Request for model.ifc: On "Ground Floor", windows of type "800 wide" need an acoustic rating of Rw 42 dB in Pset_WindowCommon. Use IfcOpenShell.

First a look at what the model holds.

```python
import ifcopenshell
import ifcopenshell.util.element

model = ifcopenshell.open("model.ifc")
print(model.schema)
storey = next(s for s in model.by_type("IfcBuildingStorey") if s.Name == "Ground Floor")
windows = [e for e in ifcopenshell.util.element.get_decomposition(storey) if e.is_a("IfcWindow")]
seen = {}
for e in windows:
    element_type = ifcopenshell.util.element.get_type(e)
    key = (element_type.Name if element_type != e and element_type else None, ifcopenshell.util.element.get_pset(e, "Pset_WindowCommon", "AcousticRating"))
    seen[key] = seen.get(key, 0) + 1
for (name, value), count in sorted(seen.items(), key=str):
    print(count, "x", name, "|", value)
```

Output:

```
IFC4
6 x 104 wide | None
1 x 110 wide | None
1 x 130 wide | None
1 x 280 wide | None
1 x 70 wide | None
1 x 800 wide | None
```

```python
import ifcopenshell
import ifcopenshell.api.pset
import ifcopenshell.util.element

model = ifcopenshell.open("model.ifc")

storey = next(s for s in model.by_type("IfcBuildingStorey") if s.Name == "Ground Floor")
windows = [e for e in ifcopenshell.util.element.get_decomposition(storey) if e.is_a("IfcWindow")]

count = 0
for e in windows:
    element_type = ifcopenshell.util.element.get_type(e)
    if element_type in (None, e) or element_type.Name != "800 wide":
        continue
    # add_pset returns the element's existing set when there is one.
    pset = ifcopenshell.api.pset.add_pset(model, product=e, name="Pset_WindowCommon")
    ifcopenshell.api.pset.edit_pset(model, pset=pset, properties={"AcousticRating": "Rw 42 dB"})
    count += 1

print(count, "windows updated")

model.write("model_updated.ifc")
```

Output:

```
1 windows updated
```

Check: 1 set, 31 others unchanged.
